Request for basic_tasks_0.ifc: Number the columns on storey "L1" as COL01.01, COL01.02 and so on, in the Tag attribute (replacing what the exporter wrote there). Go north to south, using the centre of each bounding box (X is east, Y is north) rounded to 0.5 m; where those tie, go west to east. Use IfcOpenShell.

First a look at what the model holds.

```python
import ifcopenshell
import ifcopenshell.util.element
import ifcopenshell.util.placement

model = ifcopenshell.open("basic_tasks_0.ifc")
print(model.schema)
storey = next(s for s in model.by_type("IfcBuildingStorey") if s.Name == "L1")
columns = [e for e in ifcopenshell.util.element.get_decomposition(storey) if e.is_a("IfcColumn")]
for e in sorted(columns, key=lambda e: e.id()):
    origin = ifcopenshell.util.placement.get_local_placement(e.ObjectPlacement)[:3, 3]
    print(e.id(), e.Tag, e.Name, origin.round(2) + 0.0, sep=" | ")
```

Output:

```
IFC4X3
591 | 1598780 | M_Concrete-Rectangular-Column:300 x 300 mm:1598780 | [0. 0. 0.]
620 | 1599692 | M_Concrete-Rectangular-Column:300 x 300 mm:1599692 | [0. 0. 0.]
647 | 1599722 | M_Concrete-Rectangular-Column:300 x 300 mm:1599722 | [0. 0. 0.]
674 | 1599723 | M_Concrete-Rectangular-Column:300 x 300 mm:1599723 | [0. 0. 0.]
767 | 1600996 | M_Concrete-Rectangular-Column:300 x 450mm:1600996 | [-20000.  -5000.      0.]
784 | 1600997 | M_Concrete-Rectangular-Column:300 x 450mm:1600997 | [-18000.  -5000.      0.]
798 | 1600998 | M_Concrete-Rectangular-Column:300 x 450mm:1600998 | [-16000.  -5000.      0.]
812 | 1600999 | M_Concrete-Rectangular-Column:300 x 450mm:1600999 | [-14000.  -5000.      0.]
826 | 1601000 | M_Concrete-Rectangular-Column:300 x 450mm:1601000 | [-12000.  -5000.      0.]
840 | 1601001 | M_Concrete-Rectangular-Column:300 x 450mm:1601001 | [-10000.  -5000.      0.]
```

```python
import ifcopenshell
import ifcopenshell.geom
import ifcopenshell.util.element
import ifcopenshell.util.shape

model = ifcopenshell.open("basic_tasks_0.ifc")
settings = ifcopenshell.geom.settings()
settings.set("use-world-coords", True)


def centre(element):
    shape = ifcopenshell.geom.create_shape(settings, element)
    return ifcopenshell.util.shape.get_bbox_centroid(shape.geometry)


storey = next(s for s in model.by_type("IfcBuildingStorey") if s.Name == "L1")
columns = [e for e in ifcopenshell.util.element.get_decomposition(storey) if e.is_a("IfcColumn")]

# Insertion points can sit at a corner or the storey origin, so sort by the geometry (in metres).
centres = {e: centre(e) for e in columns}
columns.sort(key=lambda e: (-round(centres[e][1] / 0.5), centres[e][0]))

for i, e in enumerate(columns, start=1):
    number = f"COL01.{i:02d}"
    e.Tag = number
    print(e.id(), number)

model.write("basic_tasks_0_edited.ifc")
```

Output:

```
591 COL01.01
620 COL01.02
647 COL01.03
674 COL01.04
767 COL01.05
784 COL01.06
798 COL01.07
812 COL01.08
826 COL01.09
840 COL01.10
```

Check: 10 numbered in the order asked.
